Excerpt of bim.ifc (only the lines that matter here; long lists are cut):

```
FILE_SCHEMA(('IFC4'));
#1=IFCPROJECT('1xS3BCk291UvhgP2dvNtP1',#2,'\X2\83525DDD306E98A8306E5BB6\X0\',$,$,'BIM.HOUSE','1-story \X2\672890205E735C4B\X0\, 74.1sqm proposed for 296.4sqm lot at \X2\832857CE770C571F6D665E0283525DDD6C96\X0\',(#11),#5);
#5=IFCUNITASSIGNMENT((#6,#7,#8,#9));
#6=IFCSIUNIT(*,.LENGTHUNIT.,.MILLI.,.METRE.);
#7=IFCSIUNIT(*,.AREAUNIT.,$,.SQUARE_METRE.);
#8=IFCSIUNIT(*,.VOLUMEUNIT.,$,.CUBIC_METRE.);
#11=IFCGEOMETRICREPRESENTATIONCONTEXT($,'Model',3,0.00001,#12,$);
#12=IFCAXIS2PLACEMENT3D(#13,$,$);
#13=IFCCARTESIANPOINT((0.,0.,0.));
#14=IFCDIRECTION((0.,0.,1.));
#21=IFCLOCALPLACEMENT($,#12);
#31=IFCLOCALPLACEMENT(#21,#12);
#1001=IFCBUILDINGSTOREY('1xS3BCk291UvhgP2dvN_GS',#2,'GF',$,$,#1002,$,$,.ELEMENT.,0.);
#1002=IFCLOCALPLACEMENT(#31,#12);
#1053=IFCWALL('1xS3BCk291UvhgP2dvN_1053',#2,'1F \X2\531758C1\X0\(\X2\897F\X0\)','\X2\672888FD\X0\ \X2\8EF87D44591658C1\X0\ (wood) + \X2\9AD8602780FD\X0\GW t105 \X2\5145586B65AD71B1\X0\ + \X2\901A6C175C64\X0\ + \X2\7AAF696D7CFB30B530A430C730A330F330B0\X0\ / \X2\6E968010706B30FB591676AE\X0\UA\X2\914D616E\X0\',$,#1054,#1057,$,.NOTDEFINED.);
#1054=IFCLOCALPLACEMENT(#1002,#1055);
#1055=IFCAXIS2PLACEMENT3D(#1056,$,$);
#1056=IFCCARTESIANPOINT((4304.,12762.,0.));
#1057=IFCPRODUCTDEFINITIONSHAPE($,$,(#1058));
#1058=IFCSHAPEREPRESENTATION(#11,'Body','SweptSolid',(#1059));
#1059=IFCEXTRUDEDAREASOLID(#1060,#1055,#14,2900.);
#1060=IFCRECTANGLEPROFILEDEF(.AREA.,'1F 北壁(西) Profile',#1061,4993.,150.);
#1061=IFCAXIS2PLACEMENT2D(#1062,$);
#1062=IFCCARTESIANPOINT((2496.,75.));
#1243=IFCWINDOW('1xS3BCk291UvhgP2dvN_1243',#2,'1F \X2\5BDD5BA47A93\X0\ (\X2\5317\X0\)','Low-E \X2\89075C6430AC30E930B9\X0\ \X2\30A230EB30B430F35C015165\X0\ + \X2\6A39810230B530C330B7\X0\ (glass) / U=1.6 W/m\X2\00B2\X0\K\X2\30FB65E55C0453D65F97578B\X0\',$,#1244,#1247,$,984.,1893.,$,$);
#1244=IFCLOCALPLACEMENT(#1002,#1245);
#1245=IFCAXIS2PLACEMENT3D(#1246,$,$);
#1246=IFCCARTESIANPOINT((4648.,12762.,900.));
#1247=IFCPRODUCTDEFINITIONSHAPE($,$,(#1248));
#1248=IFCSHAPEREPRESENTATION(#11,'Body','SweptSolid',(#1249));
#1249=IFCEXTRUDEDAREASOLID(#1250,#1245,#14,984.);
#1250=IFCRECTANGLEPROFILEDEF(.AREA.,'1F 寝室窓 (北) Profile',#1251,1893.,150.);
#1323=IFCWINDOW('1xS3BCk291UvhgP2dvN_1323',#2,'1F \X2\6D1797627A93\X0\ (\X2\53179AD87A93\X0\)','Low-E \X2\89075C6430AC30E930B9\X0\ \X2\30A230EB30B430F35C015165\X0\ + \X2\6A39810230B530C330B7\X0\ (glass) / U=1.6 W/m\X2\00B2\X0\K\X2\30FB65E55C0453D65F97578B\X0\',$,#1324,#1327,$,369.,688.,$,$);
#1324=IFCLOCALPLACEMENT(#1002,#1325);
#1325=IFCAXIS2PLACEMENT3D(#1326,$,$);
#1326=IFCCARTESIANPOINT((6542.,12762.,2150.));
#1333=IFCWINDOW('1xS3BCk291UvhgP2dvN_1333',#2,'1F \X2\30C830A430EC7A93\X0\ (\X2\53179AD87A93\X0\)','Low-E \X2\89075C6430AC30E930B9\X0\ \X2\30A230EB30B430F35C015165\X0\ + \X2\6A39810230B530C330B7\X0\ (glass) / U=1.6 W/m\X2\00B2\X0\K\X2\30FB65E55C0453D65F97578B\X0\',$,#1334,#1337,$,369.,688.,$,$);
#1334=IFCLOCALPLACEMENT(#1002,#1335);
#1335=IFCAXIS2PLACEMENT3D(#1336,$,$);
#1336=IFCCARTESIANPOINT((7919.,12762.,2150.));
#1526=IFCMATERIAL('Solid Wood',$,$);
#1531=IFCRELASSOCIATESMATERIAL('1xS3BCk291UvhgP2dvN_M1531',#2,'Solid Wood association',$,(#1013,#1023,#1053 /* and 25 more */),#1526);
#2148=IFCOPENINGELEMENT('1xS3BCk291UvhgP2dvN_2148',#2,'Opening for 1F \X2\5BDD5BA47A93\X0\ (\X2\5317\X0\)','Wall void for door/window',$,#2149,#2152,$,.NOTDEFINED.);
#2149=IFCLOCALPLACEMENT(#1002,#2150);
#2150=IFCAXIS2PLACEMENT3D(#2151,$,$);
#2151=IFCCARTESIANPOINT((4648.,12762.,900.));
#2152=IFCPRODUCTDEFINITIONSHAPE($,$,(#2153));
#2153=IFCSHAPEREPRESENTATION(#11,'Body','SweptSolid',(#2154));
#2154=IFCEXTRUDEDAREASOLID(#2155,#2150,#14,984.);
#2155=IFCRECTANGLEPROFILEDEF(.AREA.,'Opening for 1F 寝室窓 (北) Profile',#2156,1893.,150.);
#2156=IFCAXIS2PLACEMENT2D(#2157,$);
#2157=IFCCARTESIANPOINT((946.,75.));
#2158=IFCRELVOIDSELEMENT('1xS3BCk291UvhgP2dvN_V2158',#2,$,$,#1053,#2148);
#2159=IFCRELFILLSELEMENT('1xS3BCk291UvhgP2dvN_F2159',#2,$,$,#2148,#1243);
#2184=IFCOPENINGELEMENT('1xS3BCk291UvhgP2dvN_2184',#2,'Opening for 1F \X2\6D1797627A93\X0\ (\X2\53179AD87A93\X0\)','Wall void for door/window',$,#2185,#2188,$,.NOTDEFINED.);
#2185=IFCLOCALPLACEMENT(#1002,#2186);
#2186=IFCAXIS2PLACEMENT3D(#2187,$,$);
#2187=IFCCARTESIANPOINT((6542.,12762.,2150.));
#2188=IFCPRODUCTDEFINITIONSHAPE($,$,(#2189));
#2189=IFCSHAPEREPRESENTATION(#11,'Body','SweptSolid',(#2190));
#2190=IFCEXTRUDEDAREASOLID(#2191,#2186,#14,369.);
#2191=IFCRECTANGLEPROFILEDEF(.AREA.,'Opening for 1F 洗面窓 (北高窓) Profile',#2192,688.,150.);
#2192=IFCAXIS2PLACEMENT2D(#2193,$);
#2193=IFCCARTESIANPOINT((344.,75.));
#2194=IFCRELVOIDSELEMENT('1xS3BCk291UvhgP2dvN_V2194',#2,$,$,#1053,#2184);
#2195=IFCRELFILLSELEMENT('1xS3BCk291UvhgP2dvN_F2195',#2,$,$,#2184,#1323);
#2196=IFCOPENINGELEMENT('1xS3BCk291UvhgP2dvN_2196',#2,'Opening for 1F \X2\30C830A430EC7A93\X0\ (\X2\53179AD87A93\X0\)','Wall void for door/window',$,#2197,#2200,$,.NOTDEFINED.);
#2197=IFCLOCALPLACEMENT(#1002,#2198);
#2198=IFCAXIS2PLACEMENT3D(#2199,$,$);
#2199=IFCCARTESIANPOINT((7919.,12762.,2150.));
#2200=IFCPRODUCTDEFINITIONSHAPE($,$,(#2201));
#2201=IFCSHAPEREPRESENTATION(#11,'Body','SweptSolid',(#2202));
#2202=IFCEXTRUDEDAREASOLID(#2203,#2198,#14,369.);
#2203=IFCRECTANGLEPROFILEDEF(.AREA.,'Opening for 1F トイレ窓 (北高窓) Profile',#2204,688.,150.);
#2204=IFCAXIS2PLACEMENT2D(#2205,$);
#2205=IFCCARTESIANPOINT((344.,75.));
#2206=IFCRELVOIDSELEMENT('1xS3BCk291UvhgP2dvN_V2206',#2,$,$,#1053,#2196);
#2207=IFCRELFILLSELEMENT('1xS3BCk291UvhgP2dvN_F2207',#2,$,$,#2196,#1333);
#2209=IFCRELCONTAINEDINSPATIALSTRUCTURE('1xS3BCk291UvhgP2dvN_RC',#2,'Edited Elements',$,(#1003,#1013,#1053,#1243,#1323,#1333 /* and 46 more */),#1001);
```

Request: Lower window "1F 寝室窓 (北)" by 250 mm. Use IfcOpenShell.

```python
import numpy as np
import ifcopenshell
import ifcopenshell.api.geometry
import ifcopenshell.util.placement
import ifcopenshell.util.unit

model = ifcopenshell.open("bim.ifc")
unit_scale = ifcopenshell.util.unit.calculate_unit_scale(model)

window = model.by_guid("1xS3BCk291UvhgP2dvN_1243")
opening = window.FillsVoids[0].RelatingOpeningElement
dz = -0.25 / unit_scale

shift = np.array([0.0, 0.0, dz])
# The window is not placed relative to its opening, so move both.
for product in (opening, window):
    matrix = ifcopenshell.util.placement.get_local_placement(product.ObjectPlacement)
    matrix[:3, 3] += shift
    ifcopenshell.api.geometry.edit_object_placement(model, product=product, matrix=matrix, is_si=False)

print(f"moved by {dz * unit_scale:+.3f} m")

model.write("bim_rev.ifc")
```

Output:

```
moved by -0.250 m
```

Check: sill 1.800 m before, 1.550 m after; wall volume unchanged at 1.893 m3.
